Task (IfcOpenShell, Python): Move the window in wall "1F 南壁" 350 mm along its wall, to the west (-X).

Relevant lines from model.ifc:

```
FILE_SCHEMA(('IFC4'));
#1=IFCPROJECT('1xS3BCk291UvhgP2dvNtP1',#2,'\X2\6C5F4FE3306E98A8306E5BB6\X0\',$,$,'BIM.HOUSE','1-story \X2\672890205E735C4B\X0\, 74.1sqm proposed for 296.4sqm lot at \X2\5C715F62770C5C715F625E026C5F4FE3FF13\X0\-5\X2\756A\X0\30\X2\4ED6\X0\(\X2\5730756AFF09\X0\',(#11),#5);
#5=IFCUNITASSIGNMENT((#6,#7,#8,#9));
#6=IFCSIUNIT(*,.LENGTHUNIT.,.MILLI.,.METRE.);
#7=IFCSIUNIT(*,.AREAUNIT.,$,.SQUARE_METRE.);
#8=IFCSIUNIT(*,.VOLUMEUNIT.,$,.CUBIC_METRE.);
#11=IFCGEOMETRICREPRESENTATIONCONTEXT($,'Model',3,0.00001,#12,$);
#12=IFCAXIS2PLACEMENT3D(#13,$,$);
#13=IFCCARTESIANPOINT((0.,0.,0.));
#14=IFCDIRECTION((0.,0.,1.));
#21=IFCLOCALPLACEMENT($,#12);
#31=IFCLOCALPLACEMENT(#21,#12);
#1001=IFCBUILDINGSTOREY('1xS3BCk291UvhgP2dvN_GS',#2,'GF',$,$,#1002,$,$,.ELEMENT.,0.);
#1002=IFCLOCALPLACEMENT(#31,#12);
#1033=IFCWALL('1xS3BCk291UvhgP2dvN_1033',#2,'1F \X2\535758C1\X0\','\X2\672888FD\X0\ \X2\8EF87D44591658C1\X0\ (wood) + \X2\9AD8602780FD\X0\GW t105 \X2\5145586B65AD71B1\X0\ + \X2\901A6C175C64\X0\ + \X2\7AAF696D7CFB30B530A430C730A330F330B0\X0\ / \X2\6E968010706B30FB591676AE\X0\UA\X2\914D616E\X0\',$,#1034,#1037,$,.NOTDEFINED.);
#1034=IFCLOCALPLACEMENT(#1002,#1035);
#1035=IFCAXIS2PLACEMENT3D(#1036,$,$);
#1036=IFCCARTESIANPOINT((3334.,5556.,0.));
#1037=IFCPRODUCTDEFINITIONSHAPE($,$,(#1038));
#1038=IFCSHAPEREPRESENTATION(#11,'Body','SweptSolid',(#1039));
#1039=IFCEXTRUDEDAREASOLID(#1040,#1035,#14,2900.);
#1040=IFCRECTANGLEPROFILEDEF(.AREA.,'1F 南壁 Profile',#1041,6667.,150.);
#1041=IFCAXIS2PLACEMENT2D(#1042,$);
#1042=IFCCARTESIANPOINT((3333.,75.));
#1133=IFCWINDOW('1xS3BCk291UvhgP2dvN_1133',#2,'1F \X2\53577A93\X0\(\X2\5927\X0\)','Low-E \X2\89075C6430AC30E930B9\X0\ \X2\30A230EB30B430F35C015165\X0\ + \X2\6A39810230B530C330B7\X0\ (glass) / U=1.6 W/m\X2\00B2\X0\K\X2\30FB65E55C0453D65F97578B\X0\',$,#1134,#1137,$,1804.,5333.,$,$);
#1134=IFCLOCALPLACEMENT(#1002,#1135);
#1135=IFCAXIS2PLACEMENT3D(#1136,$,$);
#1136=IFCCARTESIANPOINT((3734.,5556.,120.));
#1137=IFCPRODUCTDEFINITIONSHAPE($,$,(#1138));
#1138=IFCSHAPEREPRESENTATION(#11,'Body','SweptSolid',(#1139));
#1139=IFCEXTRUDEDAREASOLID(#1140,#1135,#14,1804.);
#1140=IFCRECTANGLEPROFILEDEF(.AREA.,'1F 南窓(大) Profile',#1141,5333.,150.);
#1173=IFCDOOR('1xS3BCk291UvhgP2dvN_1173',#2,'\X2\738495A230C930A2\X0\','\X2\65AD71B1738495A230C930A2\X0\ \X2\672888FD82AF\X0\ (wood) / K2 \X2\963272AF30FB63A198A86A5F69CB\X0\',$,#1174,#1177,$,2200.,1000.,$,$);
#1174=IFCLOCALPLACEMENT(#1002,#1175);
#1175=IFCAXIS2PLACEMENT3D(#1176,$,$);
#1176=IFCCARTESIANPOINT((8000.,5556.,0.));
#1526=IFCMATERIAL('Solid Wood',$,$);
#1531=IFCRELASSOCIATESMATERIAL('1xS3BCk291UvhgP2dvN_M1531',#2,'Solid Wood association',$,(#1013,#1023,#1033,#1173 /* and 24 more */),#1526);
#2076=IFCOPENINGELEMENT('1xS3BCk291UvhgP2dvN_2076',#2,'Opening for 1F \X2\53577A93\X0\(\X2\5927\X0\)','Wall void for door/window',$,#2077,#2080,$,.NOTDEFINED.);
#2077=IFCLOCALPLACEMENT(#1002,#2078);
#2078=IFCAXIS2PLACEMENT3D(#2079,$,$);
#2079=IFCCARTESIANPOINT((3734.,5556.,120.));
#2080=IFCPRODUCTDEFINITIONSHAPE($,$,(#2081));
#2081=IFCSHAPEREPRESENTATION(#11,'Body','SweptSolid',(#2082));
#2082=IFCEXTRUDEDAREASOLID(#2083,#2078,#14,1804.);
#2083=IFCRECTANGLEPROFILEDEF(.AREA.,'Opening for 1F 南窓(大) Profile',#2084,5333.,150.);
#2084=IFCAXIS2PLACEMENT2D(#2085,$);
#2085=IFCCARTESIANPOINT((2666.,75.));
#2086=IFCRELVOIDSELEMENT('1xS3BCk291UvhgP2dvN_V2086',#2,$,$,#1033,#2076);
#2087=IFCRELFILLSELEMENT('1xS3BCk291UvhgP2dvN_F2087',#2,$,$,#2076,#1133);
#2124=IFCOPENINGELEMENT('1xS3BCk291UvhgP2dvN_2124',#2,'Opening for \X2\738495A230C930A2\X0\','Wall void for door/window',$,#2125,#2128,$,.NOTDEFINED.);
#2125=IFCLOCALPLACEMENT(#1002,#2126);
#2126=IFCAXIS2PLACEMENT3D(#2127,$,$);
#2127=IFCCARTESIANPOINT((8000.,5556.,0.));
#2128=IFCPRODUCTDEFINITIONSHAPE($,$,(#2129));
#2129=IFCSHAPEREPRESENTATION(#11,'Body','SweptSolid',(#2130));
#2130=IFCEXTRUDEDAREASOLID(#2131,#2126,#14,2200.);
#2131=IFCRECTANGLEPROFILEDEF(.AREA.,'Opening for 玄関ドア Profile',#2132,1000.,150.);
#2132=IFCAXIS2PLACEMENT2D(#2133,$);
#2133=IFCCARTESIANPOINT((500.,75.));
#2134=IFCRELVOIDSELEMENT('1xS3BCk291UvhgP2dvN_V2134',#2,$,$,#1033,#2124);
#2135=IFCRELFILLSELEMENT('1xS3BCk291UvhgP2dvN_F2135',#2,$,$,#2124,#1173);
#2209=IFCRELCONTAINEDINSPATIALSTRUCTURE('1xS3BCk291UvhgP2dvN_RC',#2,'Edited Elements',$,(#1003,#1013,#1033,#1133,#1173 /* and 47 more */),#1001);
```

```python
import ifcopenshell
import ifcopenshell.api.geometry
import ifcopenshell.util.placement

model = ifcopenshell.open("model.ifc")

window = model.by_id(1133)
opening = window.FillsVoids[0].RelatingOpeningElement
wall = opening.VoidsElements[0].RelatingBuildingElement

wall_matrix = ifcopenshell.util.placement.get_local_placement(wall.ObjectPlacement)
shift = wall_matrix[:3, 0] * -350.0
before = ifcopenshell.util.placement.get_local_placement(window.ObjectPlacement)[:3, 3].copy()

# The window is not placed relative to its opening, so move both.
for product in (opening, window):
    matrix = ifcopenshell.util.placement.get_local_placement(product.ObjectPlacement)
    matrix[:3, 3] += shift
    ifcopenshell.api.geometry.edit_object_placement(model, product=product, matrix=matrix, is_si=False)

after = ifcopenshell.util.placement.get_local_placement(window.ObjectPlacement)[:3, 3]
print("window moved by", (after - before).round(3) + 0.0)

model.write("model_edited.ifc")
```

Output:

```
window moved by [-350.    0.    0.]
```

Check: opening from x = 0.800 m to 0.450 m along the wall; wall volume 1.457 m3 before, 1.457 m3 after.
